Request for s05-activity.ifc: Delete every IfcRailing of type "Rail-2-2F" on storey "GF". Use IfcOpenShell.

First a look at what the model holds.

```python
import ifcopenshell
import ifcopenshell.util.element

model = ifcopenshell.open("s05-activity.ifc")
print(model.schema)
storey = next(s for s in model.by_type("IfcBuildingStorey") if s.Name == "GF")
railings = [e for e in ifcopenshell.util.element.get_decomposition(storey) if e.is_a("IfcRailing")]
seen = {}
for e in railings:
    element_type = ifcopenshell.util.element.get_type(e)
    name = element_type.Name if element_type not in (None, e) else None
    seen[name] = seen.get(name, 0) + 1
for name, count in sorted(seen.items(), key=str):
    print(count, "x", name)
```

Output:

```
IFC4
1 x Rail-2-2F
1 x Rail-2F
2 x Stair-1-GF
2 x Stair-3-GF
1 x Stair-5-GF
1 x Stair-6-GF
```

```python
import ifcopenshell
import ifcopenshell.api.root
import ifcopenshell.util.element

model = ifcopenshell.open("s05-activity.ifc")

storey = next(s for s in model.by_type("IfcBuildingStorey") if s.Name == "GF")
railings = [e for e in ifcopenshell.util.element.get_decomposition(storey) if e.is_a("IfcRailing")]
targets = [e for e in railings if (t := ifcopenshell.util.element.get_type(e)) not in (None, e) and t.Name == "Rail-2-2F"]

for e in targets:
    ifcopenshell.api.root.remove_product(model, product=e)
print(len(targets), "removed")

model.write("s05-activity-out.ifc")
```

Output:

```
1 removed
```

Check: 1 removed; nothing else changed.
